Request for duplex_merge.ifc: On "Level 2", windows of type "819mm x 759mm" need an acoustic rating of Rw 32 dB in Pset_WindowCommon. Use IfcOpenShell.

First a look at what the model holds.

```python
import ifcopenshell
import ifcopenshell.util.element

model = ifcopenshell.open("duplex_merge.ifc")
print(model.schema)
storey = next(s for s in model.by_type("IfcBuildingStorey") if s.Name == "Level 2")
windows = [e for e in ifcopenshell.util.element.get_decomposition(storey) if e.is_a("IfcWindow")]
seen = {}
for e in windows:
    element_type = ifcopenshell.util.element.get_type(e)
    key = (element_type.Name if element_type != e and element_type else None, ifcopenshell.util.element.get_pset(e, "Pset_WindowCommon", "AcousticRating"))
    seen[key] = seen.get(key, 0) + 1
for (name, value), count in sorted(seen.items(), key=str):
    print(count, "x", name, "|", value)
```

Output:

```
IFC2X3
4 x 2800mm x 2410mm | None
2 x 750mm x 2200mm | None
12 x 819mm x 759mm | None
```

```python
import ifcopenshell
import ifcopenshell.api.pset
import ifcopenshell.util.element

model = ifcopenshell.open("duplex_merge.ifc")

storey = next(s for s in model.by_type("IfcBuildingStorey") if s.Name == "Level 2")
windows = [e for e in ifcopenshell.util.element.get_decomposition(storey) if e.is_a("IfcWindow")]

count = 0
for e in windows:
    element_type = ifcopenshell.util.element.get_type(e)
    if element_type in (None, e) or element_type.Name != "819mm x 759mm":
        continue
    # add_pset returns the element's existing set when there is one.
    pset = ifcopenshell.api.pset.add_pset(model, product=e, name="Pset_WindowCommon")
    ifcopenshell.api.pset.edit_pset(model, pset=pset, properties={"AcousticRating": "Rw 32 dB"})
    count += 1

print(count, "windows updated")

model.write("duplex_merge_updated.ifc")
```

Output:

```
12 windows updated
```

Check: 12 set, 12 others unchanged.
